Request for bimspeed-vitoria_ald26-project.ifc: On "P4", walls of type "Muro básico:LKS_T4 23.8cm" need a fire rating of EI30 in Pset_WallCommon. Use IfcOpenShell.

First a look at what the model holds.

```python
import ifcopenshell
import ifcopenshell.util.element

model = ifcopenshell.open("bimspeed-vitoria_ald26-project.ifc")
print(model.schema)
storey = next(s for s in model.by_type("IfcBuildingStorey") if s.Name == "P4")
walls = [e for e in ifcopenshell.util.element.get_decomposition(storey) if e.is_a("IfcWall")]
seen = {}
for e in walls:
    element_type = ifcopenshell.util.element.get_type(e)
    key = (element_type.Name if element_type != e and element_type else None, ifcopenshell.util.element.get_pset(e, "Pset_WallCommon", "FireRating"))
    seen[key] = seen.get(key, 0) + 1
for (name, value), count in sorted(seen.items(), key=str):
    print(count, "x", name, "|", value)
```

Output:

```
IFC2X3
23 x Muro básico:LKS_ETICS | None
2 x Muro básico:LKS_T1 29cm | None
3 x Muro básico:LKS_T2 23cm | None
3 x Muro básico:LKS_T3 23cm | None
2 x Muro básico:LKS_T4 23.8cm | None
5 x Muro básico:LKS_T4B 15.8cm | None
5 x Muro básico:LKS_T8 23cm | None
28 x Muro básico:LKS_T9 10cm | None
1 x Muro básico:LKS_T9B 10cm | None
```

```python
import ifcopenshell
import ifcopenshell.api.pset
import ifcopenshell.util.element

model = ifcopenshell.open("bimspeed-vitoria_ald26-project.ifc")

storey = next(s for s in model.by_type("IfcBuildingStorey") if s.Name == "P4")
walls = [e for e in ifcopenshell.util.element.get_decomposition(storey) if e.is_a("IfcWall")]

count = 0
for e in walls:
    element_type = ifcopenshell.util.element.get_type(e)
    if element_type in (None, e) or element_type.Name != "Muro básico:LKS_T4 23.8cm":
        continue
    # add_pset returns the element's existing set when there is one.
    pset = ifcopenshell.api.pset.add_pset(model, product=e, name="Pset_WallCommon")
    ifcopenshell.api.pset.edit_pset(model, pset=pset, properties={"FireRating": "EI30"})
    count += 1

print(count, "walls updated")

model.write("bimspeed-vitoria_ald26-project_edited.ifc")
```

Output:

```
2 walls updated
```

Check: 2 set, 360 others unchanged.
